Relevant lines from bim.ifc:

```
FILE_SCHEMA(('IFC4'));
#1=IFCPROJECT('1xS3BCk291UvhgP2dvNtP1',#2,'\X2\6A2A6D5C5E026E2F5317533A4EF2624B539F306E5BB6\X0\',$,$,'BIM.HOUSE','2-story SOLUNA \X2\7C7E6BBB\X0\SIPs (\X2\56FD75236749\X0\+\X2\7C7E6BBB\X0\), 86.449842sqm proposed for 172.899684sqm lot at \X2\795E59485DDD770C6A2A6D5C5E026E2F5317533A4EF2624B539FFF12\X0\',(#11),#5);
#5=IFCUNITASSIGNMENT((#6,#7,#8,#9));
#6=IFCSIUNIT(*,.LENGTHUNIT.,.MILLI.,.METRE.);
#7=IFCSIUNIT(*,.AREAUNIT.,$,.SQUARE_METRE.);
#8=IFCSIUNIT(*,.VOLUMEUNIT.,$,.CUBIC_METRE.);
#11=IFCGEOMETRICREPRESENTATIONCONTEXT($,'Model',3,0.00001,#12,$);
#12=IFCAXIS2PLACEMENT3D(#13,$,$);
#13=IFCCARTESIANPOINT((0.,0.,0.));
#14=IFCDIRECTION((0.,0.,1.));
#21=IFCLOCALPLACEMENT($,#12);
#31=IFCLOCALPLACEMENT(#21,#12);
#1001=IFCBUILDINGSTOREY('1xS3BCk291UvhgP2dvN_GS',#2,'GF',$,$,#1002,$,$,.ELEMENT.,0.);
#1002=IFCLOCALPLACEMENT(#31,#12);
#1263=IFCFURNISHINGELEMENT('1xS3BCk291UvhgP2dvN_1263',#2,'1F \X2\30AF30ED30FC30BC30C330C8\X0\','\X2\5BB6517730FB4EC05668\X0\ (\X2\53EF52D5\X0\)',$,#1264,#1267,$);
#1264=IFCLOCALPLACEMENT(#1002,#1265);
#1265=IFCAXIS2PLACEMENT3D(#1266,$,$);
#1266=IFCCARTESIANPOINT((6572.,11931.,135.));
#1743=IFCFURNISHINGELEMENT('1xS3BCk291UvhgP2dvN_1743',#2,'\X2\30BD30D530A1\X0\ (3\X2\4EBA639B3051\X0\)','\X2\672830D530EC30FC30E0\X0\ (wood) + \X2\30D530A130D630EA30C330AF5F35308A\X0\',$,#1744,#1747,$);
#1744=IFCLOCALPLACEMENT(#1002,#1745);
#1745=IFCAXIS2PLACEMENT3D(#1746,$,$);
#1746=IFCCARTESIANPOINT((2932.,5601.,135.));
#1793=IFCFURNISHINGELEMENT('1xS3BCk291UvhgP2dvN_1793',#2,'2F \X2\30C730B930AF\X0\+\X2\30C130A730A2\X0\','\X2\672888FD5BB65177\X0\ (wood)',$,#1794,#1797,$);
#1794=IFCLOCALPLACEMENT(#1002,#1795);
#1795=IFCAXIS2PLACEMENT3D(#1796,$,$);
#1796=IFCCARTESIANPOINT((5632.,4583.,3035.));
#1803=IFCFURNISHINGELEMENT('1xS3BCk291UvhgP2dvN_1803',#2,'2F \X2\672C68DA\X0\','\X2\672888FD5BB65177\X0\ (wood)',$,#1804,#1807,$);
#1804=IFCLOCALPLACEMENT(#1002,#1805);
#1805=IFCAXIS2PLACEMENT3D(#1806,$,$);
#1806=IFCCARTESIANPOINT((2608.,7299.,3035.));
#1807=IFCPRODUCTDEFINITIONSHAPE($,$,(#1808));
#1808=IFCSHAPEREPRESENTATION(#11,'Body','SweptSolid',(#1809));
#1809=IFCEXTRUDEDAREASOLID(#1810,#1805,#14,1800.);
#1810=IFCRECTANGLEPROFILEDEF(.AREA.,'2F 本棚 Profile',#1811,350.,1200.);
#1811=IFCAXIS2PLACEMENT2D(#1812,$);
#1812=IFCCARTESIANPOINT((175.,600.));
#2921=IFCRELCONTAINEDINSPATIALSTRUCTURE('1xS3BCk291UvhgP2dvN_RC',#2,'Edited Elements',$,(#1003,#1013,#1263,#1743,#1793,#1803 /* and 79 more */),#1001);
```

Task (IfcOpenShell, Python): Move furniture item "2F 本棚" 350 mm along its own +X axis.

```python
import ifcopenshell
import ifcopenshell.api.geometry
import ifcopenshell.util.placement
import ifcopenshell.util.unit

model = ifcopenshell.open("bim.ifc")
unit_scale = ifcopenshell.util.unit.calculate_unit_scale(model)

item = model.by_id(1803)
matrix = ifcopenshell.util.placement.get_local_placement(item.ObjectPlacement)
matrix[:3, 3] += matrix[:3, 0] * 0.35 / unit_scale
ifcopenshell.api.geometry.edit_object_placement(model, product=item, matrix=matrix, is_si=False)

print(ifcopenshell.util.placement.get_local_placement(item.ObjectPlacement).round(3) + 0.0)

model.write("bim_v2.ifc")
```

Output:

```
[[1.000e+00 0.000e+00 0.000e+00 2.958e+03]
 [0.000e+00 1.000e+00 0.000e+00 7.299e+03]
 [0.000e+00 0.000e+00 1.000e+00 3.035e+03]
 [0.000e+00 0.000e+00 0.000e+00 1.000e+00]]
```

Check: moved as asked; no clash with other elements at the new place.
